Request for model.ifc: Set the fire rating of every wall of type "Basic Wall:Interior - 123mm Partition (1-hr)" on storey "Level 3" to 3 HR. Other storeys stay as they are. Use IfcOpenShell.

First a look at what the model holds.

```python
import ifcopenshell
import ifcopenshell.util.element

model = ifcopenshell.open("model.ifc")
print(model.schema)
storey = next(s for s in model.by_type("IfcBuildingStorey") if s.Name == "Level 3")
walls = [e for e in ifcopenshell.util.element.get_decomposition(storey) if e.is_a("IfcWall")]
seen = {}
for e in walls:
    element_type = ifcopenshell.util.element.get_type(e)
    key = (element_type.Name if element_type != e and element_type else None, ifcopenshell.util.element.get_pset(e, "Pset_WallCommon", "FireRating"))
    seen[key] = seen.get(key, 0) + 1
for (name, value), count in sorted(seen.items(), key=str):
    print(count, "x", name, "|", value)
```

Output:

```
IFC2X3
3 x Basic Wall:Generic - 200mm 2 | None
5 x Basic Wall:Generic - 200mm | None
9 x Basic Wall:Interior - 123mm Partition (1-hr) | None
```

```python
import ifcopenshell
import ifcopenshell.api.pset
import ifcopenshell.util.element

model = ifcopenshell.open("model.ifc")

storey = next(s for s in model.by_type("IfcBuildingStorey") if s.Name == "Level 3")
walls = [e for e in ifcopenshell.util.element.get_decomposition(storey) if e.is_a("IfcWall")]

count = 0
for e in walls:
    element_type = ifcopenshell.util.element.get_type(e)
    if element_type in (None, e) or element_type.Name != "Basic Wall:Interior - 123mm Partition (1-hr)":
        continue
    # add_pset returns the element's existing set when there is one.
    pset = ifcopenshell.api.pset.add_pset(model, product=e, name="Pset_WallCommon")
    ifcopenshell.api.pset.edit_pset(model, pset=pset, properties={"FireRating": "3 HR"})
    count += 1

print(count, "walls updated")

model.write("model_updated.ifc")
```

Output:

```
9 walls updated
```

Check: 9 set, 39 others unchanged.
